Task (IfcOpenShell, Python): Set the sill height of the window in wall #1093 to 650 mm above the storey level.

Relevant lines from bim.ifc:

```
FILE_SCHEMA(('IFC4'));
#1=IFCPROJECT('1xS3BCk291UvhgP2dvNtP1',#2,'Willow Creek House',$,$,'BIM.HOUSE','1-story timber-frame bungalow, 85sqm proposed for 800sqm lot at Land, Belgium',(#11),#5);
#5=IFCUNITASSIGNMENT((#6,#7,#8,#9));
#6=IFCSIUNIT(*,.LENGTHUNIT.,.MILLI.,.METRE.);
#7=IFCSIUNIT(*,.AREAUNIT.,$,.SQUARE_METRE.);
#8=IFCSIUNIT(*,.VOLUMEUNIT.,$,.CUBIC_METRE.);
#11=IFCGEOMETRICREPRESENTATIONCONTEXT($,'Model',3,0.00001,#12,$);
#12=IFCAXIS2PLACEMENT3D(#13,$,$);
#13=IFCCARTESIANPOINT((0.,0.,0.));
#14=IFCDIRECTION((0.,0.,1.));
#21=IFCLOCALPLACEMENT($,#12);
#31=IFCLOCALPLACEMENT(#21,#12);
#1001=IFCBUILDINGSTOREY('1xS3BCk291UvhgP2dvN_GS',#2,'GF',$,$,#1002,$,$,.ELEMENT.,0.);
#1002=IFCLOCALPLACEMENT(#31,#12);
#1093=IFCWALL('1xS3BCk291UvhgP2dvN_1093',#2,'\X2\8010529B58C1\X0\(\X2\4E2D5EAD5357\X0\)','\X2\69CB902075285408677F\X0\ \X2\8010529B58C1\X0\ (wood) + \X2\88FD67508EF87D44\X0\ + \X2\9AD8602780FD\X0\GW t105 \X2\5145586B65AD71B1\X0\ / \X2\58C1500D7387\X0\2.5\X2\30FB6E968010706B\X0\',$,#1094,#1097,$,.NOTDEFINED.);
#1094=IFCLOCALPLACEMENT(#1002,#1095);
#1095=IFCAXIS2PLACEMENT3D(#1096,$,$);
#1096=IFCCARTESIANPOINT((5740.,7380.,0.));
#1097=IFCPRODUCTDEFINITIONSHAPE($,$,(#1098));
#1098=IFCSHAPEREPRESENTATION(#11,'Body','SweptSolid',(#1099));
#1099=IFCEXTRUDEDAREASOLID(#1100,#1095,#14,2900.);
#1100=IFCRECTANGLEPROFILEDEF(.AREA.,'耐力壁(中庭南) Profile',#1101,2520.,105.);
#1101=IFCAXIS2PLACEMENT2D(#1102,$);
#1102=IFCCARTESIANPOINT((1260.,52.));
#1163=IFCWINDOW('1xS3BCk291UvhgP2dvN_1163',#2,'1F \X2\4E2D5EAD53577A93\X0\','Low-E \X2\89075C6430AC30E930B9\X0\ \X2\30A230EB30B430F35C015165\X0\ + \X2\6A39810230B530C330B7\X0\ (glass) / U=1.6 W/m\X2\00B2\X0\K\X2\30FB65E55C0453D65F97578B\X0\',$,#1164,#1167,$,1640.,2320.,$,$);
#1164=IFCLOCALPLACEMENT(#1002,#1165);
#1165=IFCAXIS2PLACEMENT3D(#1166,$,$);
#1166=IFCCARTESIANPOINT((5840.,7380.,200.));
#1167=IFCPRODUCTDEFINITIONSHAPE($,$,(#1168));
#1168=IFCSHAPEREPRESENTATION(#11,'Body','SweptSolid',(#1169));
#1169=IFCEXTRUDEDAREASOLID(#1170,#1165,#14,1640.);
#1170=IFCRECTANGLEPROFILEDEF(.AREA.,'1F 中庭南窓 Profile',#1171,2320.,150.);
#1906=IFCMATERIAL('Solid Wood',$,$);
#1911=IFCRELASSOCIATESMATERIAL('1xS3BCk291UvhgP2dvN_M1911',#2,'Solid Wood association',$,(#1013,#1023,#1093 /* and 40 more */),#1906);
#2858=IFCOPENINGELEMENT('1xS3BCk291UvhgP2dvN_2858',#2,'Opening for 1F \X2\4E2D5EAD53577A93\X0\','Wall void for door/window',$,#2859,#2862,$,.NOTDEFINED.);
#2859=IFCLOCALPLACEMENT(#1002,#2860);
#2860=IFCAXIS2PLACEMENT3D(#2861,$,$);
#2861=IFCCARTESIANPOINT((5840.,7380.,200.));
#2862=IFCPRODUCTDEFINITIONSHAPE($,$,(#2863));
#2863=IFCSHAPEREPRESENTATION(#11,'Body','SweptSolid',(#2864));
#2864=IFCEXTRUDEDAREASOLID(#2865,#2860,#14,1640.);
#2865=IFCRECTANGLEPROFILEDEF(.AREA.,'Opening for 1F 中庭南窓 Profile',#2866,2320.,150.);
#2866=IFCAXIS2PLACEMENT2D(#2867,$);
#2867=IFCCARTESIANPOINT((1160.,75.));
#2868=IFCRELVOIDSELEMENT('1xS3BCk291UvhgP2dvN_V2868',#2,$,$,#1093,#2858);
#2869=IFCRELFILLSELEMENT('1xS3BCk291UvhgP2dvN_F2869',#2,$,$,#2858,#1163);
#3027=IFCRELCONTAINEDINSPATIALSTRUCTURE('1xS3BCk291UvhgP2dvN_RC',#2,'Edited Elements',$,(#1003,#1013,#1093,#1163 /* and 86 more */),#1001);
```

```python
import numpy as np
import ifcopenshell
import ifcopenshell.api.geometry
import ifcopenshell.geom
import ifcopenshell.util.element
import ifcopenshell.util.placement
import ifcopenshell.util.shape
import ifcopenshell.util.unit

model = ifcopenshell.open("bim.ifc")
unit_scale = ifcopenshell.util.unit.calculate_unit_scale(model)

window = model.by_guid("1xS3BCk291UvhgP2dvN_1163")
opening = window.FillsVoids[0].RelatingOpeningElement
storey = ifcopenshell.util.element.get_container(window, ifc_class="IfcBuildingStorey")
level = ifcopenshell.util.placement.get_local_placement(storey.ObjectPlacement)[2, 3]

# The opening's origin need not be at the sill, so measure its lowest point.
shape = ifcopenshell.geom.create_shape(ifcopenshell.geom.settings(), opening)
bottom = ifcopenshell.util.shape.get_shape_bottom_elevation(shape, shape.geometry) / unit_scale
dz = level + 0.65 / unit_scale - bottom

shift = np.array([0.0, 0.0, dz])
# The window is not placed relative to its opening, so move both.
for product in (opening, window):
    matrix = ifcopenshell.util.placement.get_local_placement(product.ObjectPlacement)
    matrix[:3, 3] += shift
    ifcopenshell.api.geometry.edit_object_placement(model, product=product, matrix=matrix, is_si=False)

print(f"moved by {dz * unit_scale:+.3f} m")

model.write("bim-out.ifc")
```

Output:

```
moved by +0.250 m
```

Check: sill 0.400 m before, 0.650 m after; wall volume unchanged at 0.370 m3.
